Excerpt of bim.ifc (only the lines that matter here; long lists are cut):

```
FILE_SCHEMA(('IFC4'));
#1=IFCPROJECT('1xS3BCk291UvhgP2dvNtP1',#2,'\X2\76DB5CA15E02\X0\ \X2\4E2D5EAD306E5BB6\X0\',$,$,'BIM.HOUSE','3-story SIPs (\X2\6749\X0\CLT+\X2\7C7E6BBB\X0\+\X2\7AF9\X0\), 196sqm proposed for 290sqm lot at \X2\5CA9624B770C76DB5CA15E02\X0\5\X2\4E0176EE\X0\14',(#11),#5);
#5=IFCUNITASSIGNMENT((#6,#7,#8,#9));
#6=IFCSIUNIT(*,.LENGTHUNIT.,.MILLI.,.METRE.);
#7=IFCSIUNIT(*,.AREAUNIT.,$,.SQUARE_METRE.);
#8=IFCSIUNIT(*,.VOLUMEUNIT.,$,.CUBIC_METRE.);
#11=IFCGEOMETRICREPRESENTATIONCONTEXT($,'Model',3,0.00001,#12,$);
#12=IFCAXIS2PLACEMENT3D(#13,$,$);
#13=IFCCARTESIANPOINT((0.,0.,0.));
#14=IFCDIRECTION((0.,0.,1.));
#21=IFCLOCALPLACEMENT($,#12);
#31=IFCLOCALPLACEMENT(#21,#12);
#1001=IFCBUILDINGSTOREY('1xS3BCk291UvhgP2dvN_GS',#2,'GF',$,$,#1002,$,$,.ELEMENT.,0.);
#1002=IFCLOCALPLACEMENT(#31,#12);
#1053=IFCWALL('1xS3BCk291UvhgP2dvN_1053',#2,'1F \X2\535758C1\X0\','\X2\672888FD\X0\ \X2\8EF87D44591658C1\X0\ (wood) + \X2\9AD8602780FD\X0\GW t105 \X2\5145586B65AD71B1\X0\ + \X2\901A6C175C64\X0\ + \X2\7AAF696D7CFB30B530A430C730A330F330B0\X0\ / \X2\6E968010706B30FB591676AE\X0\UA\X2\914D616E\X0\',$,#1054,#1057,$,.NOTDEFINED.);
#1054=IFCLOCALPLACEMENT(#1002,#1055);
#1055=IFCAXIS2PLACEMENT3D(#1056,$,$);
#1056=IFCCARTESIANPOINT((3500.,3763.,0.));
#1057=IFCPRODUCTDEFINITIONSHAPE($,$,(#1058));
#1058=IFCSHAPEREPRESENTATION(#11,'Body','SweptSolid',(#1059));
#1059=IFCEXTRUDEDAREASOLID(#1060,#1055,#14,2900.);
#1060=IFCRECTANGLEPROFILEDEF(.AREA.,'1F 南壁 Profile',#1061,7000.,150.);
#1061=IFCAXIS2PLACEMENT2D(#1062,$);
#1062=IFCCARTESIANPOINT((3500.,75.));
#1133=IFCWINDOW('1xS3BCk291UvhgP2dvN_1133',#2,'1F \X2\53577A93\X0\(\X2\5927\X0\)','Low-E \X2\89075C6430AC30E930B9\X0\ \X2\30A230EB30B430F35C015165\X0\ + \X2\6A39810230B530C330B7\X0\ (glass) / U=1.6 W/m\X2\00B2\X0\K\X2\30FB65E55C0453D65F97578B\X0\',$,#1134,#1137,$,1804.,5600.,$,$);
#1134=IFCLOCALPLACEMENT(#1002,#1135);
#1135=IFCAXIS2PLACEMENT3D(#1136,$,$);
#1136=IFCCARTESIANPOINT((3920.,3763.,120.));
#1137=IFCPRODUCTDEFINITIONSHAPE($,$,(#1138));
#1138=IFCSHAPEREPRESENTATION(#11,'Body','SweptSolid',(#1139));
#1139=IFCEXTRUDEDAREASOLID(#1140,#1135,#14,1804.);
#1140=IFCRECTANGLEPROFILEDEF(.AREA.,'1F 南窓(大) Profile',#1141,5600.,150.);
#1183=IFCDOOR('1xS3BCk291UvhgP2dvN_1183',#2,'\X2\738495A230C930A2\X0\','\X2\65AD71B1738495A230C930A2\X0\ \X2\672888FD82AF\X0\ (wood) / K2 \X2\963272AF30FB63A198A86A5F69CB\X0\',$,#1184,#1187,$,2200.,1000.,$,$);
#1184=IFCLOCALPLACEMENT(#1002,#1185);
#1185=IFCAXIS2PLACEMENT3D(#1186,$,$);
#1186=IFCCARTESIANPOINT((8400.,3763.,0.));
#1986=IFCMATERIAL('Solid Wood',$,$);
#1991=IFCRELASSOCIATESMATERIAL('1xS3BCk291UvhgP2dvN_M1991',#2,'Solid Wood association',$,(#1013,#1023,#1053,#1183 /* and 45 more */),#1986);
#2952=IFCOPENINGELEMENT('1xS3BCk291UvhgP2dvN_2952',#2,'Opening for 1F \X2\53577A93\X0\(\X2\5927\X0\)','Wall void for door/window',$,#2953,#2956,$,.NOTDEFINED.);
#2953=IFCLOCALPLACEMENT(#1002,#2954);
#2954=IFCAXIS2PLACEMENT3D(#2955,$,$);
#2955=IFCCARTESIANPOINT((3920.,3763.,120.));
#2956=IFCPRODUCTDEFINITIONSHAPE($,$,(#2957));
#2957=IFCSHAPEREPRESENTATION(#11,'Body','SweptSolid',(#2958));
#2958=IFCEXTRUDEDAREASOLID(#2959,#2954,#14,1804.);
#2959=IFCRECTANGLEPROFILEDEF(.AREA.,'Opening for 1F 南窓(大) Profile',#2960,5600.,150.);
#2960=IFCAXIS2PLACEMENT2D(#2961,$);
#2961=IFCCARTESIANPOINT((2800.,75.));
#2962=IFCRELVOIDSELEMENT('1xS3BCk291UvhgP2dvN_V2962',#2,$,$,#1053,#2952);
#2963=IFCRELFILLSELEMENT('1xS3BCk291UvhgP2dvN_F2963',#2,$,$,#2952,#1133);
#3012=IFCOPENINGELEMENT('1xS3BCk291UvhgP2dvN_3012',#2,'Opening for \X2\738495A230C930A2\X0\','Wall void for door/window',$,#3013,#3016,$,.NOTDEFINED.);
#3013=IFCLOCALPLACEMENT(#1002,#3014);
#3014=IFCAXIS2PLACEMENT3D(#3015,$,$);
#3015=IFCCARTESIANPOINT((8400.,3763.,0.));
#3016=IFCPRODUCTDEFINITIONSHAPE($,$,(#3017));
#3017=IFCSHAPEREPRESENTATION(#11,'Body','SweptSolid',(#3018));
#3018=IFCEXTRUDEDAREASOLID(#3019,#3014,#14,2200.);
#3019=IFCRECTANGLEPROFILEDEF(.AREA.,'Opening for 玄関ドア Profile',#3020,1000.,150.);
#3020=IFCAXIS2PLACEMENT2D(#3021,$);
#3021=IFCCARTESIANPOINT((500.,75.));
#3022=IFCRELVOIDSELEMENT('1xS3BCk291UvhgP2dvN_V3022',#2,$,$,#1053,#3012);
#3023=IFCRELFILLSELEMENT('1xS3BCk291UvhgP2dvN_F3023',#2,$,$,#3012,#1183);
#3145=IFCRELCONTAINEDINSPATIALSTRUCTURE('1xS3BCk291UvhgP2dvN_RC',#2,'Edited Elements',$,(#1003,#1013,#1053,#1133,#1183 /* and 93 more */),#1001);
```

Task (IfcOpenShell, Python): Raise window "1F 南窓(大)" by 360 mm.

```python
import numpy as np
import ifcopenshell
import ifcopenshell.api.geometry
import ifcopenshell.util.placement
import ifcopenshell.util.unit

model = ifcopenshell.open("bim.ifc")
unit_scale = ifcopenshell.util.unit.calculate_unit_scale(model)

window = model.by_id(1133)
opening = window.FillsVoids[0].RelatingOpeningElement
dz = 0.36 / unit_scale

shift = np.array([0.0, 0.0, dz])
# The window is not placed relative to its opening, so move both.
for product in (opening, window):
    matrix = ifcopenshell.util.placement.get_local_placement(product.ObjectPlacement)
    matrix[:3, 3] += shift
    ifcopenshell.api.geometry.edit_object_placement(model, product=product, matrix=matrix, is_si=False)

print(f"moved by {dz * unit_scale:+.3f} m")

model.write("bim_edited.ifc")
```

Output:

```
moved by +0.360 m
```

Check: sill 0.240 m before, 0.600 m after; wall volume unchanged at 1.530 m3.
